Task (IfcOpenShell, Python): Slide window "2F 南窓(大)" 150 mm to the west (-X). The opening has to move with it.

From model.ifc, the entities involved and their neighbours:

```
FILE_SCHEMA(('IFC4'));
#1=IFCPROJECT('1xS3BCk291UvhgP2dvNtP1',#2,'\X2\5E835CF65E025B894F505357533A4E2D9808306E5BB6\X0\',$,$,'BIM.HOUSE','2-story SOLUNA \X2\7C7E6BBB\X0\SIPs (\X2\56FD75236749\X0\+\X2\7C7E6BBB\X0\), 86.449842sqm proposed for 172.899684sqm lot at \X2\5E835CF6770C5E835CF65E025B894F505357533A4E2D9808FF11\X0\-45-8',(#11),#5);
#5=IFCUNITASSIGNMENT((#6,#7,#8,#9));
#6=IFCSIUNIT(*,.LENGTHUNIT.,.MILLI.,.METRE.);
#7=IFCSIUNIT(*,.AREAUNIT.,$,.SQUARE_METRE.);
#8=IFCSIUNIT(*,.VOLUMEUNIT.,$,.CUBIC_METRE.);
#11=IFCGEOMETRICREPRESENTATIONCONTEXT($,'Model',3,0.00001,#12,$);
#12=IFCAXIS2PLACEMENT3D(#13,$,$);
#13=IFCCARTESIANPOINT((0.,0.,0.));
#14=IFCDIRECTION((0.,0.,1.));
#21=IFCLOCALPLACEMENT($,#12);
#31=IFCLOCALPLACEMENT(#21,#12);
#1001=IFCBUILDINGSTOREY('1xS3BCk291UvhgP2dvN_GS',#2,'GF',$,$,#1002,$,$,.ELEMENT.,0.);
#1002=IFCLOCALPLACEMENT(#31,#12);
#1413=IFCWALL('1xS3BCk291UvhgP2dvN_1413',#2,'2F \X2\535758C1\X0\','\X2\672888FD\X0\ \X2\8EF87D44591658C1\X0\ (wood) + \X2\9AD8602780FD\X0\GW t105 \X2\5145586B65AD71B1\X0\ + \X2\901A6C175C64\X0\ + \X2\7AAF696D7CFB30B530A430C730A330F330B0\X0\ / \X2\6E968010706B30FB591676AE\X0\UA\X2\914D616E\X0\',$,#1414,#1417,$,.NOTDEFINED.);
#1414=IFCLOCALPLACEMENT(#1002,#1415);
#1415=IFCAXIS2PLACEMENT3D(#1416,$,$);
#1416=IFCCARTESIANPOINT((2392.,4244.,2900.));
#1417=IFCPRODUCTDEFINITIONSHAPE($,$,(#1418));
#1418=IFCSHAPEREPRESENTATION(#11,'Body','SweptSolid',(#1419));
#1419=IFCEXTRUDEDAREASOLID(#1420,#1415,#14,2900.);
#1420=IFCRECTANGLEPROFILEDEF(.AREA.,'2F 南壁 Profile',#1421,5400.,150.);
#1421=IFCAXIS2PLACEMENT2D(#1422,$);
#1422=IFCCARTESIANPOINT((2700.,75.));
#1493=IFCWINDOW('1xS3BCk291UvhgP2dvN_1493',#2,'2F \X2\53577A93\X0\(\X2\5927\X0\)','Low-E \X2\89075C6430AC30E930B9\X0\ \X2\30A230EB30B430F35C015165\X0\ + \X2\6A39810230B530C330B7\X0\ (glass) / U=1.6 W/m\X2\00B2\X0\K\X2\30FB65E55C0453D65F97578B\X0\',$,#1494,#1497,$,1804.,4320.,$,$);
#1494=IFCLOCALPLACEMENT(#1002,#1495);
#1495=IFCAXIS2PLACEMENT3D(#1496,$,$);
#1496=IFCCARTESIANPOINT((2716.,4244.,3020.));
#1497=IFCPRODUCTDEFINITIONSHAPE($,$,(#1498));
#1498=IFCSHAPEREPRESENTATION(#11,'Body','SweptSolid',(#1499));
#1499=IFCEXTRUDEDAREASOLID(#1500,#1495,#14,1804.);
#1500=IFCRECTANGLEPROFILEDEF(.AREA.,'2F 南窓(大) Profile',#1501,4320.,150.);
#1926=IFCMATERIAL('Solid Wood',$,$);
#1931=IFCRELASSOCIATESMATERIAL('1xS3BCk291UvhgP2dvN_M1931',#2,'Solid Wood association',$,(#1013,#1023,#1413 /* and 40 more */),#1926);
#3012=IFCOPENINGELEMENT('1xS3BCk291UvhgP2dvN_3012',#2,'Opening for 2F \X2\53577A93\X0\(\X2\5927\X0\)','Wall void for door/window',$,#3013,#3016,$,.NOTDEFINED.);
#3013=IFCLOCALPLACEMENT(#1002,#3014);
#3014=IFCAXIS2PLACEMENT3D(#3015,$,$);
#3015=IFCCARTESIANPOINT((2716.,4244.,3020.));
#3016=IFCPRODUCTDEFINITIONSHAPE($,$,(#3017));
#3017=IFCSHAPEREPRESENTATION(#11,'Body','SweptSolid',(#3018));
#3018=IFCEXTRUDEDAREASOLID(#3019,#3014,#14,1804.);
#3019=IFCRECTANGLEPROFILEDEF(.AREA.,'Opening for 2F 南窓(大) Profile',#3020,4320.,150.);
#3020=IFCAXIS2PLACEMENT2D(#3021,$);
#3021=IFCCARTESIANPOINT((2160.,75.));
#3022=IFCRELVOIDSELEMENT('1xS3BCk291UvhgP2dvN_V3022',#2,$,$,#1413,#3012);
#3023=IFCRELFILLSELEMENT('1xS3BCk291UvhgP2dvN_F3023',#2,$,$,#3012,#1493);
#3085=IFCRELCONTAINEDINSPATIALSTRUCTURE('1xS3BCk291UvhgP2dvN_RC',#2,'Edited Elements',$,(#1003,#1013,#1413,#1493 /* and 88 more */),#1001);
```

```python
import ifcopenshell
import ifcopenshell.api.geometry
import ifcopenshell.util.placement
import ifcopenshell.util.unit

model = ifcopenshell.open("model.ifc")
unit_scale = ifcopenshell.util.unit.calculate_unit_scale(model)

window = model.by_id(1493)
opening = window.FillsVoids[0].RelatingOpeningElement
wall = opening.VoidsElements[0].RelatingBuildingElement

wall_matrix = ifcopenshell.util.placement.get_local_placement(wall.ObjectPlacement)
shift = wall_matrix[:3, 0] * -0.15 / unit_scale
before = ifcopenshell.util.placement.get_local_placement(window.ObjectPlacement)[:3, 3].copy()

# The window is not placed relative to its opening, so move both.
for product in (opening, window):
    matrix = ifcopenshell.util.placement.get_local_placement(product.ObjectPlacement)
    matrix[:3, 3] += shift
    ifcopenshell.api.geometry.edit_object_placement(model, product=product, matrix=matrix, is_si=False)

after = ifcopenshell.util.placement.get_local_placement(window.ObjectPlacement)[:3, 3]
print("window moved by", (after - before).round(3) + 0.0)

model.write("model_updated.ifc")
```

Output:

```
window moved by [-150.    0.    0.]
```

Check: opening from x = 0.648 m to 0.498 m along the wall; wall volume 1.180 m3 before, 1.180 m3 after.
